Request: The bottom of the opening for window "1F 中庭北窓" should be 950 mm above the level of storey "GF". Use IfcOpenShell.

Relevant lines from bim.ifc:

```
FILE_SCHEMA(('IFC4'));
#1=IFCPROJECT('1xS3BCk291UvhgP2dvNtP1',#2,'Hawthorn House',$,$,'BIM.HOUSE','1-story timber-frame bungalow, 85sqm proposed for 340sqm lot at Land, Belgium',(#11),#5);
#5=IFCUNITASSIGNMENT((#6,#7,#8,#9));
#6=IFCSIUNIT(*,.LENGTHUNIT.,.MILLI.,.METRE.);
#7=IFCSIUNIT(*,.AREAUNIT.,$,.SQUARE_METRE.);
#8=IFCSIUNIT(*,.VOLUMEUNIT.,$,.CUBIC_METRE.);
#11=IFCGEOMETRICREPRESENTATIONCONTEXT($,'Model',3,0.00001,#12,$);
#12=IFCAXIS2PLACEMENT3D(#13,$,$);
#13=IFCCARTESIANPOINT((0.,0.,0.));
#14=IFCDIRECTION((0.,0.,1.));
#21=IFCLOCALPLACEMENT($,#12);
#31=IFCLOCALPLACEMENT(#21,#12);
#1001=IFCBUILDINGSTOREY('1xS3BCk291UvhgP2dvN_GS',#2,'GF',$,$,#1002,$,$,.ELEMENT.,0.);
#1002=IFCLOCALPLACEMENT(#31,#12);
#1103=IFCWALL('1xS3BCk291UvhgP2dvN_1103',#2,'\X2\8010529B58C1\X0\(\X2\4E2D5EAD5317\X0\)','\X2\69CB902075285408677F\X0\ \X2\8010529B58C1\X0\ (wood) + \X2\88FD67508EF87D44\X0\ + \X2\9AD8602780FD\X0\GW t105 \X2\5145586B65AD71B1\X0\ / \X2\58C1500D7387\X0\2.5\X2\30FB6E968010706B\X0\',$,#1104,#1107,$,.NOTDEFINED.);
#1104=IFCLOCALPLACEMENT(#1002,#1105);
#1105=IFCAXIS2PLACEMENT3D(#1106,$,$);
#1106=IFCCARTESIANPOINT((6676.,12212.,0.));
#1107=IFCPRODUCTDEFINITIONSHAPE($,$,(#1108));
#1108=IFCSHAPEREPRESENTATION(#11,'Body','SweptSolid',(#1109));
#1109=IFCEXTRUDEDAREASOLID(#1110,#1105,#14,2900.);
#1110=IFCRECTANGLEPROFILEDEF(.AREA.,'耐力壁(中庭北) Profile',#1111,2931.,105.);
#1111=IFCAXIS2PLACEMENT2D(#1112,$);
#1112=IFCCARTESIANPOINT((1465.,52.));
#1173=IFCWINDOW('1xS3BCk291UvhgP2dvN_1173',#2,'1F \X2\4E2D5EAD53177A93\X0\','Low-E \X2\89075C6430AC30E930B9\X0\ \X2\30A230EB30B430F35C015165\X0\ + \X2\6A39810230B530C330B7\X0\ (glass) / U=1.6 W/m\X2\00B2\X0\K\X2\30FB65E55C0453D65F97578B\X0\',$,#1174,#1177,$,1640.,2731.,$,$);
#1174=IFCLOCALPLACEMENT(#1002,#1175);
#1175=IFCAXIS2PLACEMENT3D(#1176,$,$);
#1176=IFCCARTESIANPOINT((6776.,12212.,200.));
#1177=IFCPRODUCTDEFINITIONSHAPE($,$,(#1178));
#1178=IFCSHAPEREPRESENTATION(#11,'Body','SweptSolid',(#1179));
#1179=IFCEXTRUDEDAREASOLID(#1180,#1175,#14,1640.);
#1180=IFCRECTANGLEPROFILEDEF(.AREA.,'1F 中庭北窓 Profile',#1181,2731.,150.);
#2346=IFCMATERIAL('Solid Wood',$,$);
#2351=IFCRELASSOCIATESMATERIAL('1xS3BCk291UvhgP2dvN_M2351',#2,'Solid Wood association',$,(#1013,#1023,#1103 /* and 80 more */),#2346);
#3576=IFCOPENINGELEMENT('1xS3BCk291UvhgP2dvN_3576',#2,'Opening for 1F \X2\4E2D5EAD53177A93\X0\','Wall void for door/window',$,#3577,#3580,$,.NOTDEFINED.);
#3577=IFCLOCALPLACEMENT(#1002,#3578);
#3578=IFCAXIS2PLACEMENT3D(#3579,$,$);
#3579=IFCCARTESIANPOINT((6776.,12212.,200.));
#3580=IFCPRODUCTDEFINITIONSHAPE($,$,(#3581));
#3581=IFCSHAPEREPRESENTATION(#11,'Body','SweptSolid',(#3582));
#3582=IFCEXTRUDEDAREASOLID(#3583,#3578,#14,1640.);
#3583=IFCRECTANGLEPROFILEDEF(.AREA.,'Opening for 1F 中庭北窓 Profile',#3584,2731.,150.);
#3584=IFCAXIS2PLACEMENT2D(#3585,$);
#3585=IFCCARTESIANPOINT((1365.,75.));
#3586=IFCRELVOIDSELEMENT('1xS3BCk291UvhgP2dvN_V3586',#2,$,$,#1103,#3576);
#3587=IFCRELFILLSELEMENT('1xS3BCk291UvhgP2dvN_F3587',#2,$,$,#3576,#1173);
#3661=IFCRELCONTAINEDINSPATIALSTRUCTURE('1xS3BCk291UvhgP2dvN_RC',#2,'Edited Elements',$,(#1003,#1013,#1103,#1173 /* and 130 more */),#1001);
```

```python
import numpy as np
import ifcopenshell
import ifcopenshell.api.geometry
import ifcopenshell.geom
import ifcopenshell.util.element
import ifcopenshell.util.placement
import ifcopenshell.util.shape
import ifcopenshell.util.unit

model = ifcopenshell.open("bim.ifc")
unit_scale = ifcopenshell.util.unit.calculate_unit_scale(model)

window = model.by_guid("1xS3BCk291UvhgP2dvN_1173")
opening = window.FillsVoids[0].RelatingOpeningElement
storey = ifcopenshell.util.element.get_container(window, ifc_class="IfcBuildingStorey")
level = ifcopenshell.util.placement.get_local_placement(storey.ObjectPlacement)[2, 3]

# The opening's origin need not be at the sill, so measure its lowest point.
shape = ifcopenshell.geom.create_shape(ifcopenshell.geom.settings(), opening)
bottom = ifcopenshell.util.shape.get_shape_bottom_elevation(shape, shape.geometry) / unit_scale
dz = level + 0.95 / unit_scale - bottom

shift = np.array([0.0, 0.0, dz])
# The window is not placed relative to its opening, so move both.
for product in (opening, window):
    matrix = ifcopenshell.util.placement.get_local_placement(product.ObjectPlacement)
    matrix[:3, 3] += shift
    ifcopenshell.api.geometry.edit_object_placement(model, product=product, matrix=matrix, is_si=False)

print(f"moved by {dz * unit_scale:+.3f} m")

model.write("bim_edited.ifc")
```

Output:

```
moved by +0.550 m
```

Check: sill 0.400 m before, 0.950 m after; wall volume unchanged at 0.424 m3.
